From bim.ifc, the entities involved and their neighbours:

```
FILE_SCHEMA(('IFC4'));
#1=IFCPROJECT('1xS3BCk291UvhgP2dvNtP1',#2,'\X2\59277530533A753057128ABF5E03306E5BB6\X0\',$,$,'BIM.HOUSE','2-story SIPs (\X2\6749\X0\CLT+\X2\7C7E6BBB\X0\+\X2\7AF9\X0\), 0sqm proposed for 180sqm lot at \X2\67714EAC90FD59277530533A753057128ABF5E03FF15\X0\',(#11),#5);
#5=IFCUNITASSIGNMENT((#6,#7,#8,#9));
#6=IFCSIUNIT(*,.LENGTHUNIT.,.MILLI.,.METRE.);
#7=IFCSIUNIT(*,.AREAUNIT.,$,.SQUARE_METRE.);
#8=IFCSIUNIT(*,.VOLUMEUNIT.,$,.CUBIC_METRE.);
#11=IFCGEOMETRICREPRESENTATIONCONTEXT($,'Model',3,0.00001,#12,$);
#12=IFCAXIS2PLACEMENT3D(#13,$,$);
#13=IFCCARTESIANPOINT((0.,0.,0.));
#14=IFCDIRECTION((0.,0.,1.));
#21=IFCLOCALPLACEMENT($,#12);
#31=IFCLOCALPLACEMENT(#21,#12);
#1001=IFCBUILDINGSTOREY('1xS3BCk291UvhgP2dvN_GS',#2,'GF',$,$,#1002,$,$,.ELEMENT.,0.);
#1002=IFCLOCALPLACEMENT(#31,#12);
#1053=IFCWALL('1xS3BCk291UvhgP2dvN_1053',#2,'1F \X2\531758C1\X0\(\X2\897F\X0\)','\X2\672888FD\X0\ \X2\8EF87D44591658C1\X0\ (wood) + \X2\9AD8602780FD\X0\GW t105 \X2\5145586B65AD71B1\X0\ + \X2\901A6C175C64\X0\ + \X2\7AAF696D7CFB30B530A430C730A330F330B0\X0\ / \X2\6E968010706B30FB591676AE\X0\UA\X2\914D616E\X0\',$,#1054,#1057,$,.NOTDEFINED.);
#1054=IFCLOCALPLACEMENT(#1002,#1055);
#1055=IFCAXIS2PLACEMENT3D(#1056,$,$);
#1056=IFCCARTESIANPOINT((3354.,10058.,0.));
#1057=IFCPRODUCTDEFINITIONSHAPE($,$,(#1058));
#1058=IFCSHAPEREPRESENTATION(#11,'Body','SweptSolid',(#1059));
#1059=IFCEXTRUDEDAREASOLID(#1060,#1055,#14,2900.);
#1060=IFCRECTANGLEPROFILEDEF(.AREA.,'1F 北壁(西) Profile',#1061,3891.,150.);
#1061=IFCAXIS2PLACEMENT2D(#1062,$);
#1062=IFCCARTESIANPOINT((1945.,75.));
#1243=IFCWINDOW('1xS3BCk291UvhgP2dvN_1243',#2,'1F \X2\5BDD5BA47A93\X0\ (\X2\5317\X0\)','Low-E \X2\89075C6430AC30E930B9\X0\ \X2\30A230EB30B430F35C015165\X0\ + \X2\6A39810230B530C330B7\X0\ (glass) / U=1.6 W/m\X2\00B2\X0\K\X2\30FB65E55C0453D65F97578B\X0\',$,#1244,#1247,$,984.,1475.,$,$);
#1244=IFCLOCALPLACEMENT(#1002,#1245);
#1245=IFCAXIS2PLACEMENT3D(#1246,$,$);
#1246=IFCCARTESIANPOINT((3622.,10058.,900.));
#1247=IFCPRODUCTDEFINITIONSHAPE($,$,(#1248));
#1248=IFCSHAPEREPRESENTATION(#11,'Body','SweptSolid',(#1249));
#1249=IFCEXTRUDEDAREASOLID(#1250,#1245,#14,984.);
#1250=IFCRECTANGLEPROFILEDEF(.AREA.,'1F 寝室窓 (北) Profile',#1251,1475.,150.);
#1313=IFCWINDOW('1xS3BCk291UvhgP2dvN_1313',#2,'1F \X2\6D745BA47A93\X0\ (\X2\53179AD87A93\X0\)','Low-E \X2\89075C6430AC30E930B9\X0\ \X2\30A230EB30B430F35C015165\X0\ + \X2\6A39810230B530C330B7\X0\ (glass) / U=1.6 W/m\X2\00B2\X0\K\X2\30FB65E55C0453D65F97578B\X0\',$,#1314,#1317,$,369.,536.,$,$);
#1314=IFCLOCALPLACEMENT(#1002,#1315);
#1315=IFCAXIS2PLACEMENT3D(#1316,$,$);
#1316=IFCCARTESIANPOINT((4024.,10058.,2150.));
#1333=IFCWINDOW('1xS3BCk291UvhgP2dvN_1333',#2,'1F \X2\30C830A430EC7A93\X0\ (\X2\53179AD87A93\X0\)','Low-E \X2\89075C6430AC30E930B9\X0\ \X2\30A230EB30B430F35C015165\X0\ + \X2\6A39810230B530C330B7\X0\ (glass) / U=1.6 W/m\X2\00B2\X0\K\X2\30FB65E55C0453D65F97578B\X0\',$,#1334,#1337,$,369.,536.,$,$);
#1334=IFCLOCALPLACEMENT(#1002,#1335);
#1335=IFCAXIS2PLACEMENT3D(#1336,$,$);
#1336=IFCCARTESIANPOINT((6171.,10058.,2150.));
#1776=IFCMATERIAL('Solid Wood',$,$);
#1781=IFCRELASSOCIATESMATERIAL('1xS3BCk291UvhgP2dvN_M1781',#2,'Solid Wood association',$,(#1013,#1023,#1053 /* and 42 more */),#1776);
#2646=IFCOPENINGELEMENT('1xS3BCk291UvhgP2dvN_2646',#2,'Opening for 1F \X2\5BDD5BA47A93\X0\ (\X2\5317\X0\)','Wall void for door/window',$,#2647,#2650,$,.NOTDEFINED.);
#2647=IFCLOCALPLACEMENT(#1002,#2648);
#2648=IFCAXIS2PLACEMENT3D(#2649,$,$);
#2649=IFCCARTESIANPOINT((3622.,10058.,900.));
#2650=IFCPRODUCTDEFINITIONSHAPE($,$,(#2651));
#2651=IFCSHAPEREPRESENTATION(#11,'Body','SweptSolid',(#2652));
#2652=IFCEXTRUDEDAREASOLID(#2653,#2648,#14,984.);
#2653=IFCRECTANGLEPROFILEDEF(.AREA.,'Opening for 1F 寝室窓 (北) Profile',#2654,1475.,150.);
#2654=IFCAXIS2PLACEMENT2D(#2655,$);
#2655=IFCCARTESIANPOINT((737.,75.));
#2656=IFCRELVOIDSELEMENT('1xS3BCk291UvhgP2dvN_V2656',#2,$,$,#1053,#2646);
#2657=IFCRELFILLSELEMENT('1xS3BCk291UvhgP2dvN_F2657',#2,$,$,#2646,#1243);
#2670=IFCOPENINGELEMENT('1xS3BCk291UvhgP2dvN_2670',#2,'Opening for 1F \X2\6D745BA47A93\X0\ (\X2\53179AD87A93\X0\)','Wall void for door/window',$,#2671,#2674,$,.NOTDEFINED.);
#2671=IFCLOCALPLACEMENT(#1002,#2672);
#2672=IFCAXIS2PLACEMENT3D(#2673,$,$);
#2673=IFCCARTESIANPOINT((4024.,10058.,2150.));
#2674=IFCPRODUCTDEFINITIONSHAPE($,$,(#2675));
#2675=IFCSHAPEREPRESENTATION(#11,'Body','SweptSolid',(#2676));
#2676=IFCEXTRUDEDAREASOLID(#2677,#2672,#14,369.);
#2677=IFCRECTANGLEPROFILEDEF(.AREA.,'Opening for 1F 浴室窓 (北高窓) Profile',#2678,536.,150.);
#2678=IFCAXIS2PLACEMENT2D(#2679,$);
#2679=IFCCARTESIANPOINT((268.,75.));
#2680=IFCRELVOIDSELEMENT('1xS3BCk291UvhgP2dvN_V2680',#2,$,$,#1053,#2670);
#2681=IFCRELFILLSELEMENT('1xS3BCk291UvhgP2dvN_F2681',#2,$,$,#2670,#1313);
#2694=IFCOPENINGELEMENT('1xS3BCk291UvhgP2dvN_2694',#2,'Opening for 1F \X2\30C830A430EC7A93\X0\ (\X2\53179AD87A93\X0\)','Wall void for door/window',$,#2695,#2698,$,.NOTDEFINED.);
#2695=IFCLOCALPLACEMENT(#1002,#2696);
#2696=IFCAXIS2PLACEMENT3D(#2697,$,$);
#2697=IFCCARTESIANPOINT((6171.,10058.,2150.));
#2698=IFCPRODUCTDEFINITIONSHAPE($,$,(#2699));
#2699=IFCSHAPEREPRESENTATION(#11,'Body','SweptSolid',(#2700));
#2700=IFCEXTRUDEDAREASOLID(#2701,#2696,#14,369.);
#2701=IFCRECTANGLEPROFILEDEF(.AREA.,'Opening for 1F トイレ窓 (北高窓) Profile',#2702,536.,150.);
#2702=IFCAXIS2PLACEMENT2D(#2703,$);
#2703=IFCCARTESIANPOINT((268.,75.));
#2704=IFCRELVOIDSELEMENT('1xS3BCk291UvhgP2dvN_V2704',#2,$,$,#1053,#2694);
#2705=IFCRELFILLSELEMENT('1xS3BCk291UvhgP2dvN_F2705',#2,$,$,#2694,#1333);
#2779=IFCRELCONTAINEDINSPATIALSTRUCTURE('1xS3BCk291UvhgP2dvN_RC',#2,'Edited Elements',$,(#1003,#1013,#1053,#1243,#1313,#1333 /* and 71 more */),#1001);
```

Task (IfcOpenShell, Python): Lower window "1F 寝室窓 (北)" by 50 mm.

```python
import numpy as np
import ifcopenshell
import ifcopenshell.api.geometry
import ifcopenshell.util.placement
import ifcopenshell.util.unit

model = ifcopenshell.open("bim.ifc")
unit_scale = ifcopenshell.util.unit.calculate_unit_scale(model)

window = model.by_guid("1xS3BCk291UvhgP2dvN_1243")
opening = window.FillsVoids[0].RelatingOpeningElement
dz = -50.0

shift = np.array([0.0, 0.0, dz])
# The window is not placed relative to its opening, so move both.
for product in (opening, window):
    matrix = ifcopenshell.util.placement.get_local_placement(product.ObjectPlacement)
    matrix[:3, 3] += shift
    ifcopenshell.api.geometry.edit_object_placement(model, product=product, matrix=matrix, is_si=False)

print(f"moved by {dz * unit_scale:+.3f} m")

model.write("bim_rev.ifc")
```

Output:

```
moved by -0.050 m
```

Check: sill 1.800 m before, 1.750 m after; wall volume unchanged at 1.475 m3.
